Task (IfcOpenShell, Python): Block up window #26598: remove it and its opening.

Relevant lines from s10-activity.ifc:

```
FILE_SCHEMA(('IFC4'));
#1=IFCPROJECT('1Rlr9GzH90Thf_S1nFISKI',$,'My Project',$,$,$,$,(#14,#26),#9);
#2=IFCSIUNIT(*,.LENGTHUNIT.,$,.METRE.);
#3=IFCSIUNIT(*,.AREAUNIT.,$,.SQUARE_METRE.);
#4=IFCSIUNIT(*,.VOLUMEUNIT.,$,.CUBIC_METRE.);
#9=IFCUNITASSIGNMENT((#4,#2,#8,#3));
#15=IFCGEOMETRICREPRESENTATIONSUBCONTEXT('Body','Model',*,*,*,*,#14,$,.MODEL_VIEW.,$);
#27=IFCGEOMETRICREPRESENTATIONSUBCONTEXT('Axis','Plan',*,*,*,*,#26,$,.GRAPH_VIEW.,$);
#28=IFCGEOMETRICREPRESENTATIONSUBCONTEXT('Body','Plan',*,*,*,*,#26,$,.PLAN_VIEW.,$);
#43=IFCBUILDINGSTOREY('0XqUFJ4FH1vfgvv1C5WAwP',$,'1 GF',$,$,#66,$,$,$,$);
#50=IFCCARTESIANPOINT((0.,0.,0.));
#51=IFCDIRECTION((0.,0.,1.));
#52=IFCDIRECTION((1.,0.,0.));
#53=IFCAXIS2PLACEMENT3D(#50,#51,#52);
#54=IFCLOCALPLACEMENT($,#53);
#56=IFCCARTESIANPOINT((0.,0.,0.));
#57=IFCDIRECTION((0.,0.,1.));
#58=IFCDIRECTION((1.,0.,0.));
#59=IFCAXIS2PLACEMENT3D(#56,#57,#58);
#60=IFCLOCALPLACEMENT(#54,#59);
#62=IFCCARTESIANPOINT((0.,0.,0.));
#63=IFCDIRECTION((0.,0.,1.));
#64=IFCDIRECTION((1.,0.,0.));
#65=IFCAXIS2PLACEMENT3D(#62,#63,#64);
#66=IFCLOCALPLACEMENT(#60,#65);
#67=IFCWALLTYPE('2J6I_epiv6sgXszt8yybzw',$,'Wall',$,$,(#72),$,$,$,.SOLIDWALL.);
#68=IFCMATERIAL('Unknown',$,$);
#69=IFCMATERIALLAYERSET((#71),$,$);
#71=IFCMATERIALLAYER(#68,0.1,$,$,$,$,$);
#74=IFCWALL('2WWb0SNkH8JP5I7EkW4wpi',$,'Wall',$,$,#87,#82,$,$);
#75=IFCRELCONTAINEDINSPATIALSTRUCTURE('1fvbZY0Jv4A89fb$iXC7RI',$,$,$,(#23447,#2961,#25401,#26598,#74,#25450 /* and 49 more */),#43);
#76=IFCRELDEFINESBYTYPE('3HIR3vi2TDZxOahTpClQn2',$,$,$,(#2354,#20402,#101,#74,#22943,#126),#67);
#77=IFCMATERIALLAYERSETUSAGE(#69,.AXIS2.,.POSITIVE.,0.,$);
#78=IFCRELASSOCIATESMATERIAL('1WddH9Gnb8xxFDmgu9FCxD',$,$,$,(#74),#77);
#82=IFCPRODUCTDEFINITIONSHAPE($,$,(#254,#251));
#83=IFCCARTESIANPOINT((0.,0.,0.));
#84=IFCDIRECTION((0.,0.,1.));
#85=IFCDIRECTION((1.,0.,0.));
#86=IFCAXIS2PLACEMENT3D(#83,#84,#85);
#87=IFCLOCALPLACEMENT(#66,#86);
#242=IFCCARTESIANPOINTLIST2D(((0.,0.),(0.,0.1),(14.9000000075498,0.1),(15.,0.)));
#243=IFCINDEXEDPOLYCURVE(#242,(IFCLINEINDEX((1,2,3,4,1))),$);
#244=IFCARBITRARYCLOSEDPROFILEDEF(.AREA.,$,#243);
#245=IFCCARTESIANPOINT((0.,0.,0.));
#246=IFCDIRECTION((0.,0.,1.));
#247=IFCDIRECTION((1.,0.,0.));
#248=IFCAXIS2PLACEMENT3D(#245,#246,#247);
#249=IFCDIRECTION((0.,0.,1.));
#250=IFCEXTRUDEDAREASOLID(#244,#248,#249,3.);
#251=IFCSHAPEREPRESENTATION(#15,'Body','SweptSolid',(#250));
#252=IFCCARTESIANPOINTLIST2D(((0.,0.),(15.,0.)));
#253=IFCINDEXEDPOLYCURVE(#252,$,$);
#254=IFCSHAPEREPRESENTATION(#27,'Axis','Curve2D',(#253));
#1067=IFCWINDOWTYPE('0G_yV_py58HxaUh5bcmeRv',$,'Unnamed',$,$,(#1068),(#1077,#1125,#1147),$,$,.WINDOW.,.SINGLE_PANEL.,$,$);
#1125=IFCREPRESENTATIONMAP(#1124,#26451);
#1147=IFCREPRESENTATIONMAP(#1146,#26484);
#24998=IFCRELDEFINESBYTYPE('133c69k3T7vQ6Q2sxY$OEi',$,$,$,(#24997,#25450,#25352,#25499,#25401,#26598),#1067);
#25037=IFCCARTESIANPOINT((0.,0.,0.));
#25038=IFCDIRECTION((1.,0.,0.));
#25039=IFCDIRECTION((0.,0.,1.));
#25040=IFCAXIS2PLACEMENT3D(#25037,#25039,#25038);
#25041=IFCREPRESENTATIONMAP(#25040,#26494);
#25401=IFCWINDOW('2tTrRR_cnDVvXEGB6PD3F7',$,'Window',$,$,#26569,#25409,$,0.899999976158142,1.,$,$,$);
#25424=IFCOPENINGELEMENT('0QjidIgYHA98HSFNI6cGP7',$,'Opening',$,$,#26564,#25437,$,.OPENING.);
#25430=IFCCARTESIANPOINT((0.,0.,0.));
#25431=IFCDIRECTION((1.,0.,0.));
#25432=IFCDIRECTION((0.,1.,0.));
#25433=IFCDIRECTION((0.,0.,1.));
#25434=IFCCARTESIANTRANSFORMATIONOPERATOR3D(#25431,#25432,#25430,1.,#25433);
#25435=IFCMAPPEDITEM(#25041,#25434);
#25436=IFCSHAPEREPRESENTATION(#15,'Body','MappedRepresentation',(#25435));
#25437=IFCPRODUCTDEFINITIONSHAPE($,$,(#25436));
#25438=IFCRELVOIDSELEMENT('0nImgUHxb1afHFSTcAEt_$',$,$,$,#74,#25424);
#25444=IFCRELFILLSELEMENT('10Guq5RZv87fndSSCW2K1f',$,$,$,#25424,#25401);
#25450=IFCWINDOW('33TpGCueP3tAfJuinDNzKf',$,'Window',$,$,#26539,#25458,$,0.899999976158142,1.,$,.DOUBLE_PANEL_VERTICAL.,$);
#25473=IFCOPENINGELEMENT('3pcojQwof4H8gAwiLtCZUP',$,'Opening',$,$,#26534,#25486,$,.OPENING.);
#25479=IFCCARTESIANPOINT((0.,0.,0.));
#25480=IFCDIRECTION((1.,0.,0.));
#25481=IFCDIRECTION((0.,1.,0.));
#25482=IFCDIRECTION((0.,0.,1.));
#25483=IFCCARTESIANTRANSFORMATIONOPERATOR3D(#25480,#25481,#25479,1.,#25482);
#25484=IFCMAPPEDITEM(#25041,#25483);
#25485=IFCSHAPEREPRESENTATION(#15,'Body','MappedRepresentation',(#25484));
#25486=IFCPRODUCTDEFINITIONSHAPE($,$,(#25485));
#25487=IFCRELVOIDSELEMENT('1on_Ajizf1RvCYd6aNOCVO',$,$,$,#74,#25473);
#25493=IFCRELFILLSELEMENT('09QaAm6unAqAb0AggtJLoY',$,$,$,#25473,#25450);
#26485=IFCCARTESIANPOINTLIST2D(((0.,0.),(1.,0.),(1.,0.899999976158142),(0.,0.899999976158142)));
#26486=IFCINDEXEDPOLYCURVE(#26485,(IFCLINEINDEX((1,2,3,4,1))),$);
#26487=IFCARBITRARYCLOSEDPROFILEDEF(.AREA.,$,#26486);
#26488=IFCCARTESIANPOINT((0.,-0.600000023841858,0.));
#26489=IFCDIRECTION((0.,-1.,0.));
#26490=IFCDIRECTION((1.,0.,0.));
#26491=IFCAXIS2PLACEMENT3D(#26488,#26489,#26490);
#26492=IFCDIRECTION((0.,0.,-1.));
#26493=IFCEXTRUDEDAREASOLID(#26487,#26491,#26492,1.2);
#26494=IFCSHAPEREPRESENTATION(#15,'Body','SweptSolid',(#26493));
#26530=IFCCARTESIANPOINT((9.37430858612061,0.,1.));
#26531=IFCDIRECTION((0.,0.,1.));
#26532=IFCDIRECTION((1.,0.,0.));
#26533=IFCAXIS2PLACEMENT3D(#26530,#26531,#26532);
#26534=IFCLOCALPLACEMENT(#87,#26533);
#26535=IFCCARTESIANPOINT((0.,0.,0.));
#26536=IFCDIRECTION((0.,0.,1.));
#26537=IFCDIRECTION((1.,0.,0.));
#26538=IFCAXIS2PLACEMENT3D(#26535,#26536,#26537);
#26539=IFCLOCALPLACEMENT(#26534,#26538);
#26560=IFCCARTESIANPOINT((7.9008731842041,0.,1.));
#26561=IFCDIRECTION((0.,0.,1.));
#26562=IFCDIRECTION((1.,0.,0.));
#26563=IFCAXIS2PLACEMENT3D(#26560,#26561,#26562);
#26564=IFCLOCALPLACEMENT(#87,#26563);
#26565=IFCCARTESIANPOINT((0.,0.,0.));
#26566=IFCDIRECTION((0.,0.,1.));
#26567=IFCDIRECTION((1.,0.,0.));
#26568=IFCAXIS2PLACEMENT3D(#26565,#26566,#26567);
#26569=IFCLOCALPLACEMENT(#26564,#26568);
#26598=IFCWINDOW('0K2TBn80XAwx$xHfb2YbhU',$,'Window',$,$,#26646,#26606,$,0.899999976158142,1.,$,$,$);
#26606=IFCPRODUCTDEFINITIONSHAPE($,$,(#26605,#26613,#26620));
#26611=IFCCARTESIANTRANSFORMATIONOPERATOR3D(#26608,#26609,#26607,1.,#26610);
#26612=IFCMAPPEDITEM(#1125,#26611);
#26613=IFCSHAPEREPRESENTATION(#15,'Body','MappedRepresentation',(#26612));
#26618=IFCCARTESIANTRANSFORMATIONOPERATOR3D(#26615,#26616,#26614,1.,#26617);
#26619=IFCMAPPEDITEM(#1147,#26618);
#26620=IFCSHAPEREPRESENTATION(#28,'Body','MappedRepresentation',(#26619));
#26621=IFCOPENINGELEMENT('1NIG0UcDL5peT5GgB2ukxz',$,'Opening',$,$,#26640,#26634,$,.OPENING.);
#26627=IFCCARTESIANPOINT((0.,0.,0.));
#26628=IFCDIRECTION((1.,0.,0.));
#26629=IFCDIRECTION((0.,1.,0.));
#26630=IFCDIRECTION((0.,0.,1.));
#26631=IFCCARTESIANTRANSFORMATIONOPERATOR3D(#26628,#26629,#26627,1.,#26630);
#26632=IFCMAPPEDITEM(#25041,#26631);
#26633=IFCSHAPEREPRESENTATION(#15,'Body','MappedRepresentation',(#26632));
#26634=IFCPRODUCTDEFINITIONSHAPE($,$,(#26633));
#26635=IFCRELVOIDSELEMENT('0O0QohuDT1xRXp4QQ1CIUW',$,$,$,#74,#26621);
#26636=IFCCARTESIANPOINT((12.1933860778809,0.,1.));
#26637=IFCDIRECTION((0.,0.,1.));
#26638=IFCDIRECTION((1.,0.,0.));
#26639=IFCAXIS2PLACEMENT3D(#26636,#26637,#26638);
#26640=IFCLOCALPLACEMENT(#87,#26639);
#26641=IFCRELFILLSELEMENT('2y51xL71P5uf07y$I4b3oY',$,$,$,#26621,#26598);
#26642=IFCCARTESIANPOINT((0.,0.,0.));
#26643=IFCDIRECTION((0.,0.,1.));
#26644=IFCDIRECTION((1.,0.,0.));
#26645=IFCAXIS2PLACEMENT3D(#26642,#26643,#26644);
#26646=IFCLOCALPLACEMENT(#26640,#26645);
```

```python
import ifcopenshell
import ifcopenshell.api.feature
import ifcopenshell.api.root
import ifcopenshell.geom
import ifcopenshell.util.shape

model = ifcopenshell.open("s10-activity.ifc")
settings = ifcopenshell.geom.settings()


def volume(element):
    """Net volume in cubic metres, openings subtracted."""
    shape = ifcopenshell.geom.create_shape(settings, element)
    return ifcopenshell.util.shape.get_volume(shape.geometry)


window = model.by_guid("0K2TBn80XAwx$xHfb2YbhU")
opening = window.FillsVoids[0].RelatingOpeningElement
wall = opening.VoidsElements[0].RelatingBuildingElement
before = volume(wall)

ifcopenshell.api.root.remove_product(model, product=window)
ifcopenshell.api.feature.remove_feature(model, feature=opening)

after = volume(wall)

print(f"wall volume {before:.3f} -> {after:.3f} m3")

model.write("s10-activity_updated.ifc")
```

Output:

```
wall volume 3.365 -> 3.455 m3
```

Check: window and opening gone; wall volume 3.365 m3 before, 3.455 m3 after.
